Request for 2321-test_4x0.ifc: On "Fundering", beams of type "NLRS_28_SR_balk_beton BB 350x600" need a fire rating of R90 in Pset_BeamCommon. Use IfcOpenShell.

First a look at what the model holds.

```python
import ifcopenshell
import ifcopenshell.util.element

model = ifcopenshell.open("2321-test_4x0.ifc")
print(model.schema)
storey = next(s for s in model.by_type("IfcBuildingStorey") if s.Name == "Fundering")
beams = [e for e in ifcopenshell.util.element.get_decomposition(storey) if e.is_a("IfcBeam")]
seen = {}
for e in beams:
    element_type = ifcopenshell.util.element.get_type(e)
    key = (element_type.Name if element_type != e and element_type else None, ifcopenshell.util.element.get_pset(e, "Pset_BeamCommon", "FireRating"))
    seen[key] = seen.get(key, 0) + 1
for (name, value), count in sorted(seen.items(), key=str):
    print(count, "x", name, "|", value)
```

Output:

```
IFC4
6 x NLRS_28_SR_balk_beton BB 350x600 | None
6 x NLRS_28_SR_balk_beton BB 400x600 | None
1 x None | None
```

```python
import ifcopenshell
import ifcopenshell.api.pset
import ifcopenshell.util.element

model = ifcopenshell.open("2321-test_4x0.ifc")

storey = next(s for s in model.by_type("IfcBuildingStorey") if s.Name == "Fundering")
beams = [e for e in ifcopenshell.util.element.get_decomposition(storey) if e.is_a("IfcBeam")]

count = 0
for e in beams:
    element_type = ifcopenshell.util.element.get_type(e)
    if element_type in (None, e) or element_type.Name != "NLRS_28_SR_balk_beton BB 350x600":
        continue
    # add_pset returns the element's existing set when there is one.
    pset = ifcopenshell.api.pset.add_pset(model, product=e, name="Pset_BeamCommon")
    ifcopenshell.api.pset.edit_pset(model, pset=pset, properties={"FireRating": "R90"})
    count += 1

print(count, "beams updated")

model.write("2321-test_4x0_v2.ifc")
```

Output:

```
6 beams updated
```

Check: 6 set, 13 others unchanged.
